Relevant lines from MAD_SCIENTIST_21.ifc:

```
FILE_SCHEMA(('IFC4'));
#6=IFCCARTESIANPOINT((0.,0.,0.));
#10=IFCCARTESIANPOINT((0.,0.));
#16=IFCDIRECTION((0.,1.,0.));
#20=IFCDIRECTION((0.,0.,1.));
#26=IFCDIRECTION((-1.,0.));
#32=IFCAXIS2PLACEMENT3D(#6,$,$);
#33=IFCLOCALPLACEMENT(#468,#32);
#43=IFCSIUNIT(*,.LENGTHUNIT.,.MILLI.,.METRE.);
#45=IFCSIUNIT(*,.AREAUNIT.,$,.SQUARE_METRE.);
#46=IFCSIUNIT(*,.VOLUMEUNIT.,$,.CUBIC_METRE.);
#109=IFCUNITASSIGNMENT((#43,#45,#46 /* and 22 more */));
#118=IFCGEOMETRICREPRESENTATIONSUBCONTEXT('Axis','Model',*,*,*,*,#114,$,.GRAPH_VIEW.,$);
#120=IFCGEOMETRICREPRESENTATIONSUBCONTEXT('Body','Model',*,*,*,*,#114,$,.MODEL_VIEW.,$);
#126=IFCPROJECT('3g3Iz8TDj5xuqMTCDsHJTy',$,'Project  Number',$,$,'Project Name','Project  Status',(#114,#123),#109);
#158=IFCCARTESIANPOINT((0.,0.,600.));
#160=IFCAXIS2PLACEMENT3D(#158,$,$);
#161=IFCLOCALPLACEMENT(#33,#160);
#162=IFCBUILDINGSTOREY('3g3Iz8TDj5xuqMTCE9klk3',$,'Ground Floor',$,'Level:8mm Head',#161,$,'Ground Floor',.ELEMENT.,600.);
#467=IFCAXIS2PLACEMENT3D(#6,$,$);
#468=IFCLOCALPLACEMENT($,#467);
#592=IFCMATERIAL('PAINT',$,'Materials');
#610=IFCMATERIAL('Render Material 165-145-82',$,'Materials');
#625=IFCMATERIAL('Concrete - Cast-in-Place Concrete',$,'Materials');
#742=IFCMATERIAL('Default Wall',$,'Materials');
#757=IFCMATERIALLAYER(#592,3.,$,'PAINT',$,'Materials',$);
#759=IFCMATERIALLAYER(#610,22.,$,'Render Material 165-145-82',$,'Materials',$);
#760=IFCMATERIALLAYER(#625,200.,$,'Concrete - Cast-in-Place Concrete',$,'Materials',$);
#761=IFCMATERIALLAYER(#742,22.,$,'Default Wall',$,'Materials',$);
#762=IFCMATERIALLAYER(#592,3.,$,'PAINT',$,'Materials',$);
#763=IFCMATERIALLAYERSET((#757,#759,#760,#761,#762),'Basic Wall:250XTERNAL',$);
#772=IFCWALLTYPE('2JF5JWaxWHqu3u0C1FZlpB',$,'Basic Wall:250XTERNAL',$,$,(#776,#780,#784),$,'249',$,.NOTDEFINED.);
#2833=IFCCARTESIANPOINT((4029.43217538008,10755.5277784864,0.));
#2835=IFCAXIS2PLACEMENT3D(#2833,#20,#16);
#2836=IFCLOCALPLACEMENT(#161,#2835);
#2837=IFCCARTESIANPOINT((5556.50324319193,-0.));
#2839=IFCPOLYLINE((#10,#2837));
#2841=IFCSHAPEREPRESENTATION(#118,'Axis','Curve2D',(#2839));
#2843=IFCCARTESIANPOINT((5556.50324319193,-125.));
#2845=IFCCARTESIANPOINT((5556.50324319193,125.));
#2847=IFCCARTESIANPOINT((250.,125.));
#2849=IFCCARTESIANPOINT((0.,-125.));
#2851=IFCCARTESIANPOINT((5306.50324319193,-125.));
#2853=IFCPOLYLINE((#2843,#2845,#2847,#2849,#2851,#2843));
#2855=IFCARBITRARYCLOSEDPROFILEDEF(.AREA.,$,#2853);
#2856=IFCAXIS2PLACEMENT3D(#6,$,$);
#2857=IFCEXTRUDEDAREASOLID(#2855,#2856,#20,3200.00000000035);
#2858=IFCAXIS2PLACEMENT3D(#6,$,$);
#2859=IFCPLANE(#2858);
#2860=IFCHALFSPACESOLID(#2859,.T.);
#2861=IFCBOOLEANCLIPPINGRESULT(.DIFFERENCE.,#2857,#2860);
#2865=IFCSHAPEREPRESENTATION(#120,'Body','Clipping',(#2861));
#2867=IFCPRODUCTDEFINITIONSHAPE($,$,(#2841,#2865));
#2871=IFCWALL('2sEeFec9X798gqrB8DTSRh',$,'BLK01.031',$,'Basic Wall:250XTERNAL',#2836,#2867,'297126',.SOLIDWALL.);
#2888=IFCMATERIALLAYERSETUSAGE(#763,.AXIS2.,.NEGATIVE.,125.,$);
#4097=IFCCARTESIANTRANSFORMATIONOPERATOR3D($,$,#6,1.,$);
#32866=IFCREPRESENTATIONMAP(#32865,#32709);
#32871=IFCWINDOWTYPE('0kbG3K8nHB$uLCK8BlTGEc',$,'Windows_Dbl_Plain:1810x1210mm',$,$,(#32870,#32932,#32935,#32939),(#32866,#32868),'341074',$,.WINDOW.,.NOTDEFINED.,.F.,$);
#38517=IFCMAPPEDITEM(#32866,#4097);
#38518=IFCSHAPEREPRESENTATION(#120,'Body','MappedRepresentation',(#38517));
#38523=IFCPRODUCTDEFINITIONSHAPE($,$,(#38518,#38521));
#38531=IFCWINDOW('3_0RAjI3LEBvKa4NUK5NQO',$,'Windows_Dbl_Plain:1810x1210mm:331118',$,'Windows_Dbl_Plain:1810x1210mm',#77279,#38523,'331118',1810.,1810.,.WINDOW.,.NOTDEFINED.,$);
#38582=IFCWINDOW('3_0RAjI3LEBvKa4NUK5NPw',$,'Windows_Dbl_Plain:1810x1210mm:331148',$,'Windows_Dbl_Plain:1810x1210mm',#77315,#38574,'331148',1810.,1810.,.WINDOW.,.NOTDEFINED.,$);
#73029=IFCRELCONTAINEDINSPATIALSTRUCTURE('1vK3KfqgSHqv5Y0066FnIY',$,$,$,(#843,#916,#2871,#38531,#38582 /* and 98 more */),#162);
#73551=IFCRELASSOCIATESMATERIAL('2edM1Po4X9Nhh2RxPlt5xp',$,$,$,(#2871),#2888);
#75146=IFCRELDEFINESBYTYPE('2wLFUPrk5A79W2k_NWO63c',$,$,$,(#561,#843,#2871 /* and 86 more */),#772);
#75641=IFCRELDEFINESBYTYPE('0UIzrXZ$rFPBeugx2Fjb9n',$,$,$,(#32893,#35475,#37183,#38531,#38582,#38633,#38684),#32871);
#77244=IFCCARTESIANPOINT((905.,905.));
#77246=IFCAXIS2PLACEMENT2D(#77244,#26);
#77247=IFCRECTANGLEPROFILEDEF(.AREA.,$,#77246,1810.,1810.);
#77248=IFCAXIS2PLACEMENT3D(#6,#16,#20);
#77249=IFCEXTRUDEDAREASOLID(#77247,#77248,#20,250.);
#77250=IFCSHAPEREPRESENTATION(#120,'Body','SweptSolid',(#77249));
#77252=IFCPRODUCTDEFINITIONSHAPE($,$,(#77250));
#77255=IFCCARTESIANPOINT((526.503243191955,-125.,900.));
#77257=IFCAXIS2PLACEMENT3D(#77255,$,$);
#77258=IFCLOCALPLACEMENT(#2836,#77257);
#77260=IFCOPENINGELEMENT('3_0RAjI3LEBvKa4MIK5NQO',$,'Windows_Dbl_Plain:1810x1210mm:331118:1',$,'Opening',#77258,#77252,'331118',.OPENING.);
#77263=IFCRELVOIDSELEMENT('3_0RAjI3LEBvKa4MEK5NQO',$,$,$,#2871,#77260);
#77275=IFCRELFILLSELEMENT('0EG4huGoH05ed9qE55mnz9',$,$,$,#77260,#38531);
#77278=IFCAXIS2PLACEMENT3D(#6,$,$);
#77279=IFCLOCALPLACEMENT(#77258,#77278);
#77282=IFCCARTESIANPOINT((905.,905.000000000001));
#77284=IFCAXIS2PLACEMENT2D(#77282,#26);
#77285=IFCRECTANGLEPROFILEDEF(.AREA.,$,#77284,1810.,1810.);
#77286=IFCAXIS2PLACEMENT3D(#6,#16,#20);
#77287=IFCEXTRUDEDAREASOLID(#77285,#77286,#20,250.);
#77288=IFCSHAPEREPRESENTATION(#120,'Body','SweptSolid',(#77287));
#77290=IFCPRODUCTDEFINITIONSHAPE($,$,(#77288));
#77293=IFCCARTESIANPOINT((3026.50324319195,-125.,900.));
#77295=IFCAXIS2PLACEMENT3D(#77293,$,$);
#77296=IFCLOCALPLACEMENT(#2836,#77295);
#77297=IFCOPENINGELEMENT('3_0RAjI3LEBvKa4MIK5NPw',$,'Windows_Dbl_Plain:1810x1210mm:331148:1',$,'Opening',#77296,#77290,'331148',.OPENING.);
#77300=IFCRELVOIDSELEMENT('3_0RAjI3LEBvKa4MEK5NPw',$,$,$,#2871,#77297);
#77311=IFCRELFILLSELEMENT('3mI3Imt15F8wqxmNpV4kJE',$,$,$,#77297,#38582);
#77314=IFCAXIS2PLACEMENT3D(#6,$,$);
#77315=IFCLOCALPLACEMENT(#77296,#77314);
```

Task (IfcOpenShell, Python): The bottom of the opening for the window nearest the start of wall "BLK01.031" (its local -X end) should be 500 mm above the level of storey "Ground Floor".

```python
import numpy as np
import ifcopenshell
import ifcopenshell.api.geometry
import ifcopenshell.geom
import ifcopenshell.util.element
import ifcopenshell.util.placement
import ifcopenshell.util.shape
import ifcopenshell.util.unit

model = ifcopenshell.open("MAD_SCIENTIST_21.ifc")
unit_scale = ifcopenshell.util.unit.calculate_unit_scale(model)

window = model.by_guid("3_0RAjI3LEBvKa4NUK5NQO")
opening = window.FillsVoids[0].RelatingOpeningElement
storey = ifcopenshell.util.element.get_container(window, ifc_class="IfcBuildingStorey")
level = ifcopenshell.util.placement.get_local_placement(storey.ObjectPlacement)[2, 3]

# The opening's origin need not be at the sill, so measure its lowest point.
shape = ifcopenshell.geom.create_shape(ifcopenshell.geom.settings(), opening)
bottom = ifcopenshell.util.shape.get_shape_bottom_elevation(shape, shape.geometry) / unit_scale
dz = level + 0.5 / unit_scale - bottom

shift = np.array([0.0, 0.0, dz])
# The window is placed relative to its opening, so it follows when the opening moves.
matrix = ifcopenshell.util.placement.get_local_placement(opening.ObjectPlacement)
matrix[:3, 3] += shift
ifcopenshell.api.geometry.edit_object_placement(
    model, product=opening, matrix=matrix, is_si=False, should_transform_children=True
)

print(f"moved by {dz * unit_scale:+.3f} m")

model.write("MAD_SCIENTIST_21_rev.ifc")
```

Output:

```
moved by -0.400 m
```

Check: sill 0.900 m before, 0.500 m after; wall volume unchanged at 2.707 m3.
